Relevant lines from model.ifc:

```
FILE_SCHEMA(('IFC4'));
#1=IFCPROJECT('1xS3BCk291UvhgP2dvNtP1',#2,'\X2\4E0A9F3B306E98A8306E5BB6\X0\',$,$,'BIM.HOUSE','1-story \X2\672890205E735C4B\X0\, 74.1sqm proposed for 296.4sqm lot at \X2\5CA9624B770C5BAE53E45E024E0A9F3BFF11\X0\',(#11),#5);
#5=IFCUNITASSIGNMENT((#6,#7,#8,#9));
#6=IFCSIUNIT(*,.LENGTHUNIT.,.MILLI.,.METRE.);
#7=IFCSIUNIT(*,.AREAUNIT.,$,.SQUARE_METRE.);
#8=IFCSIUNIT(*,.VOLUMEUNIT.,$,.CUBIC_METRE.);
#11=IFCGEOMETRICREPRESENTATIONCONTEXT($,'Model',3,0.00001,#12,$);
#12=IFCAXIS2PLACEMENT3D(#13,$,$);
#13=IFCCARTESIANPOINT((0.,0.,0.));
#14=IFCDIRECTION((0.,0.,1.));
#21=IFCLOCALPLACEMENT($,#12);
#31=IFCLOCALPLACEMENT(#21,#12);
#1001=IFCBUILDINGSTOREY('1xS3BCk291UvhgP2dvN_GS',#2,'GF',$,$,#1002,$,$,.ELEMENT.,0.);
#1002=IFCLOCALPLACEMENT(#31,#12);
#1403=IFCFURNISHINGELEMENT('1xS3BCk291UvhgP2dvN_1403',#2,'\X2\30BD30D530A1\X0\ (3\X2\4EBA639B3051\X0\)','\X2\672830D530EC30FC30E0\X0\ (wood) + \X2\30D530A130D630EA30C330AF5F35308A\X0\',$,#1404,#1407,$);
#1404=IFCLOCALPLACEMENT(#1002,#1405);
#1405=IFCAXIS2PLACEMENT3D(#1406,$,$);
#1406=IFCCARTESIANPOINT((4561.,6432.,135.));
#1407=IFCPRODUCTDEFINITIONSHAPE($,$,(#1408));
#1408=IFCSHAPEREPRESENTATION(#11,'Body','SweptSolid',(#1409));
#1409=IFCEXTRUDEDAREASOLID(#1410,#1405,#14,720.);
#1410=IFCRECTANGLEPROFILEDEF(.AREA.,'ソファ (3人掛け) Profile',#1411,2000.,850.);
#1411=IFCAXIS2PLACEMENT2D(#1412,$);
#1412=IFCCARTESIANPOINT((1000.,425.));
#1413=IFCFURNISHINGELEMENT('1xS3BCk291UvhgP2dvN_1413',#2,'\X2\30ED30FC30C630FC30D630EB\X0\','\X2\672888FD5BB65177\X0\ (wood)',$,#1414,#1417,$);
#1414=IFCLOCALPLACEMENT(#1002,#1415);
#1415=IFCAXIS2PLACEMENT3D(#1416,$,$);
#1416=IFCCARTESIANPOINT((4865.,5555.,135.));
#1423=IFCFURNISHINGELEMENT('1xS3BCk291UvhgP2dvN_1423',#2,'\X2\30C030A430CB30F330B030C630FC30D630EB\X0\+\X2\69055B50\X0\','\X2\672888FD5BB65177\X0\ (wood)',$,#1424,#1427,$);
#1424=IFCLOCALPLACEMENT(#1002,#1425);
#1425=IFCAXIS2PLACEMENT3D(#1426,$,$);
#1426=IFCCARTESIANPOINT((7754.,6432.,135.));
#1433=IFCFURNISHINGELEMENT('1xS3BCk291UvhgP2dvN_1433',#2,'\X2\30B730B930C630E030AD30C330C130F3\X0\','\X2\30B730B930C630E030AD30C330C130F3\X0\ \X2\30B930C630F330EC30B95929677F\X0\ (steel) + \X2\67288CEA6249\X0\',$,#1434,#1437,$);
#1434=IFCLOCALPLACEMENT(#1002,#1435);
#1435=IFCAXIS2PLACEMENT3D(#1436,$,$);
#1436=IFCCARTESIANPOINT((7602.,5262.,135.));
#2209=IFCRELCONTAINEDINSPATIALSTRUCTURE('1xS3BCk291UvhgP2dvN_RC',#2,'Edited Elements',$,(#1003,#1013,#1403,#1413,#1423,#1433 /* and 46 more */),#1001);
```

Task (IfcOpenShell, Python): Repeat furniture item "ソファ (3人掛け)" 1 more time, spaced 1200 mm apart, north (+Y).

```python
import numpy as np
import ifcopenshell
import ifcopenshell.api.geometry
import ifcopenshell.api.root
import ifcopenshell.util.element
import ifcopenshell.util.placement

model = ifcopenshell.open("model.ifc")


def reuse_history(source, copy):
    """copy_class also copies each property set's owner history, people and application; keep the originals."""
    for rel in copy.IsDefinedBy:
        if rel.is_a("IfcRelDefinesByProperties") and (history := rel.RelatingPropertyDefinition.OwnerHistory):
            rel.RelatingPropertyDefinition.OwnerHistory = source.OwnerHistory
            ifcopenshell.util.element.remove_deep2(model, history)


source = model.by_guid("1xS3BCk291UvhgP2dvN_1403")
base = ifcopenshell.util.placement.get_local_placement(source.ObjectPlacement)
step = np.array([0.0, 1.0, 0.0]) * 1200.0

for i in range(1, 2):
    copy = ifcopenshell.api.root.copy_class(model, product=source)
    copy.Representation = ifcopenshell.util.element.copy_deep(
        model, source.Representation, exclude=["IfcGeometricRepresentationContext", "IfcRepresentationMap"]
    )
    reuse_history(source, copy)
    matrix = base.copy()
    matrix[:3, 3] += i * step
    print("added at", matrix[:3, 3].round(3) + 0.0)
    ifcopenshell.api.geometry.edit_object_placement(model, product=copy, matrix=matrix, is_si=False)

model.write("model_edited.ifc")
```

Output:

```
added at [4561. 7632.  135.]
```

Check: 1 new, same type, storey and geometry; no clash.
